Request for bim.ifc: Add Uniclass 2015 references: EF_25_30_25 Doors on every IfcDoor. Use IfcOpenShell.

First a look at what the model holds.

```python
import ifcopenshell

model = ifcopenshell.open("bim.ifc")
print(model.schema)
print("classifications:", [c.Name for c in model.by_type("IfcClassification")])
for ifc_class in ("IfcDoor", "IfcRoof", "IfcStair", "IfcWall", "IfcWindow"):
    print(ifc_class, len(model.by_type(ifc_class)))
```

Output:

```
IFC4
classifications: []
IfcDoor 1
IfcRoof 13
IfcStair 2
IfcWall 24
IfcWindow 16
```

```python
import ifcopenshell
import ifcopenshell.api.classification

model = ifcopenshell.open("bim.ifc")

system = ifcopenshell.api.classification.add_classification(model, classification="Uniclass 2015")

codes = {
    "IfcDoor": ("EF_25_30_25", "Doors"),
}
for ifc_class, (code, name) in codes.items():
    products = model.by_type(ifc_class)
    ifcopenshell.api.classification.add_reference(
        model, products=products, classification=system, identification=code, name=name
    )
    print(code, len(products))

model.write("bim-out.ifc")
```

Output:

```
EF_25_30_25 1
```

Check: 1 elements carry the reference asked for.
